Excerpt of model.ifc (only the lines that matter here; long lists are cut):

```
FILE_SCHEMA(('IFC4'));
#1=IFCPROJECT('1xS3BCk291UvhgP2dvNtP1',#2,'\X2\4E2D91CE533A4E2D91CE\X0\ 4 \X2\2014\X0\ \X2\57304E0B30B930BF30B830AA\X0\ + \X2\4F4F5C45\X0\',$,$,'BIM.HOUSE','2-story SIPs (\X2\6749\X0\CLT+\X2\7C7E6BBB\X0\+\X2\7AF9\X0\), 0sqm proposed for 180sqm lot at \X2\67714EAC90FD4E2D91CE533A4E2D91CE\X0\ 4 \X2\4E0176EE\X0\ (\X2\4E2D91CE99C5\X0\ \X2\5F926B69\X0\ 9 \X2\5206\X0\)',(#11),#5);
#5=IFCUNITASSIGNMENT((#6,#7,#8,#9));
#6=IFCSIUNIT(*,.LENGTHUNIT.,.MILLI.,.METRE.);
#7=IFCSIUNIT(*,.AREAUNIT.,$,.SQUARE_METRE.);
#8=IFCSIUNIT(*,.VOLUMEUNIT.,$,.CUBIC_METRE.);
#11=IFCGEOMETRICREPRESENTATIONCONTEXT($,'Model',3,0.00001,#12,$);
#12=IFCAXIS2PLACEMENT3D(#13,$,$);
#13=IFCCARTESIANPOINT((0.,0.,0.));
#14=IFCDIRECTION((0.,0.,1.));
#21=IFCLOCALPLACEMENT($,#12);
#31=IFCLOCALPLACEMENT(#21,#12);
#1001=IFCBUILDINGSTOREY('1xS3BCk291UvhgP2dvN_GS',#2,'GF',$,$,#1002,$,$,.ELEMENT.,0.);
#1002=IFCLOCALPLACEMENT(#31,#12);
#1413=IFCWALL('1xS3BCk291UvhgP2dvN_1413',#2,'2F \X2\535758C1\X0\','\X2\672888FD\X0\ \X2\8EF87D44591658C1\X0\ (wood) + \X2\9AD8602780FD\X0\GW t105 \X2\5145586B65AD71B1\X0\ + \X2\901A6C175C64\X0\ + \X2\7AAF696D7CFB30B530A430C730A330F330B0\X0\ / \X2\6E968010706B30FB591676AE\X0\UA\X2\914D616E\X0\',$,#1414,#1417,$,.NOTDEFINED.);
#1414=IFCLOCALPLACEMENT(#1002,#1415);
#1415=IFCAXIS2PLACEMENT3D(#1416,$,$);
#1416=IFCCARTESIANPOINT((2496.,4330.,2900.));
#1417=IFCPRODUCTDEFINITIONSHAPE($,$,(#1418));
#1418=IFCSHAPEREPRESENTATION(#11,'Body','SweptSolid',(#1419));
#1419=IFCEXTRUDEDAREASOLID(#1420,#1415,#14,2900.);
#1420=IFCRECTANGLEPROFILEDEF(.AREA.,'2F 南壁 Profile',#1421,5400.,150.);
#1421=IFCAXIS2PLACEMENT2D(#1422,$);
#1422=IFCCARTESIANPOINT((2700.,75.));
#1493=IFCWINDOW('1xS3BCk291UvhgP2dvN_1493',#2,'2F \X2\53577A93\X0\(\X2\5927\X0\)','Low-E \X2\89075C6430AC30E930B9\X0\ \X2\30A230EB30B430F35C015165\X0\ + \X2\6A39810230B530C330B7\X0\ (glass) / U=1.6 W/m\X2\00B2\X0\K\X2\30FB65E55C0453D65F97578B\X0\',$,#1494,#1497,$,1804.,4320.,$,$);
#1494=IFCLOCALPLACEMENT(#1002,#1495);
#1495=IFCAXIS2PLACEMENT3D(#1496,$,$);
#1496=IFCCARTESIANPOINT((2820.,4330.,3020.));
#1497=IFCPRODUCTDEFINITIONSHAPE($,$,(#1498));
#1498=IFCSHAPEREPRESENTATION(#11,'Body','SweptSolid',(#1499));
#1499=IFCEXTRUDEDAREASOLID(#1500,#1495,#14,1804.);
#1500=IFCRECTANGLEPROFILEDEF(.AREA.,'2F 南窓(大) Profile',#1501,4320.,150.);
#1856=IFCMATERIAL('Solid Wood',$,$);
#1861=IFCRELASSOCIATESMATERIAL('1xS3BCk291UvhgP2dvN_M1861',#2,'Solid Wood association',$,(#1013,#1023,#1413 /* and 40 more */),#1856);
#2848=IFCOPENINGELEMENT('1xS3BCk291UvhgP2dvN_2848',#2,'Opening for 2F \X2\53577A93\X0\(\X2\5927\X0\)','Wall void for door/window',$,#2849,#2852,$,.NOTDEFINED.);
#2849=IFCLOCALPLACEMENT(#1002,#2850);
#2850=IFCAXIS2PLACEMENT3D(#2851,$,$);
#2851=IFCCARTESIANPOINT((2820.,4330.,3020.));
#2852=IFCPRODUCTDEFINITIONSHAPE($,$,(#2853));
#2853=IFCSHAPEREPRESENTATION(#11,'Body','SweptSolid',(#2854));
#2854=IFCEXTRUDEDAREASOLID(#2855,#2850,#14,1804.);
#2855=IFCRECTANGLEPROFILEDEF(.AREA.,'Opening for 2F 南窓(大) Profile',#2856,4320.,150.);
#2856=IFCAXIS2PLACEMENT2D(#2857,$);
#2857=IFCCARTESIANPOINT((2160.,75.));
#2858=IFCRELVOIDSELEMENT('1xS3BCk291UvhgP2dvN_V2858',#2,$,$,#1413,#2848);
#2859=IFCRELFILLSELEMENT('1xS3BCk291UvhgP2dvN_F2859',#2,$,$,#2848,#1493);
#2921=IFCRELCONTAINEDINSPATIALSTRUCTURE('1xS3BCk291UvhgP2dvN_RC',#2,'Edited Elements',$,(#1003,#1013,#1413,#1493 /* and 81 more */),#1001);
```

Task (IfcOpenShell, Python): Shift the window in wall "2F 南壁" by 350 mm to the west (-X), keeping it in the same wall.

```python
import ifcopenshell
import ifcopenshell.api.geometry
import ifcopenshell.util.placement

model = ifcopenshell.open("model.ifc")

window = model.by_guid("1xS3BCk291UvhgP2dvN_1493")
opening = window.FillsVoids[0].RelatingOpeningElement
wall = opening.VoidsElements[0].RelatingBuildingElement

wall_matrix = ifcopenshell.util.placement.get_local_placement(wall.ObjectPlacement)
shift = wall_matrix[:3, 0] * -350.0
before = ifcopenshell.util.placement.get_local_placement(window.ObjectPlacement)[:3, 3].copy()

# The window is not placed relative to its opening, so move both.
for product in (opening, window):
    matrix = ifcopenshell.util.placement.get_local_placement(product.ObjectPlacement)
    matrix[:3, 3] += shift
    ifcopenshell.api.geometry.edit_object_placement(model, product=product, matrix=matrix, is_si=False)

after = ifcopenshell.util.placement.get_local_placement(window.ObjectPlacement)[:3, 3]
print("window moved by", (after - before).round(3) + 0.0)

model.write("model_rev.ifc")
```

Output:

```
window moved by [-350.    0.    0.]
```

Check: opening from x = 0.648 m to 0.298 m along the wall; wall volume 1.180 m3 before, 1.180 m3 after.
